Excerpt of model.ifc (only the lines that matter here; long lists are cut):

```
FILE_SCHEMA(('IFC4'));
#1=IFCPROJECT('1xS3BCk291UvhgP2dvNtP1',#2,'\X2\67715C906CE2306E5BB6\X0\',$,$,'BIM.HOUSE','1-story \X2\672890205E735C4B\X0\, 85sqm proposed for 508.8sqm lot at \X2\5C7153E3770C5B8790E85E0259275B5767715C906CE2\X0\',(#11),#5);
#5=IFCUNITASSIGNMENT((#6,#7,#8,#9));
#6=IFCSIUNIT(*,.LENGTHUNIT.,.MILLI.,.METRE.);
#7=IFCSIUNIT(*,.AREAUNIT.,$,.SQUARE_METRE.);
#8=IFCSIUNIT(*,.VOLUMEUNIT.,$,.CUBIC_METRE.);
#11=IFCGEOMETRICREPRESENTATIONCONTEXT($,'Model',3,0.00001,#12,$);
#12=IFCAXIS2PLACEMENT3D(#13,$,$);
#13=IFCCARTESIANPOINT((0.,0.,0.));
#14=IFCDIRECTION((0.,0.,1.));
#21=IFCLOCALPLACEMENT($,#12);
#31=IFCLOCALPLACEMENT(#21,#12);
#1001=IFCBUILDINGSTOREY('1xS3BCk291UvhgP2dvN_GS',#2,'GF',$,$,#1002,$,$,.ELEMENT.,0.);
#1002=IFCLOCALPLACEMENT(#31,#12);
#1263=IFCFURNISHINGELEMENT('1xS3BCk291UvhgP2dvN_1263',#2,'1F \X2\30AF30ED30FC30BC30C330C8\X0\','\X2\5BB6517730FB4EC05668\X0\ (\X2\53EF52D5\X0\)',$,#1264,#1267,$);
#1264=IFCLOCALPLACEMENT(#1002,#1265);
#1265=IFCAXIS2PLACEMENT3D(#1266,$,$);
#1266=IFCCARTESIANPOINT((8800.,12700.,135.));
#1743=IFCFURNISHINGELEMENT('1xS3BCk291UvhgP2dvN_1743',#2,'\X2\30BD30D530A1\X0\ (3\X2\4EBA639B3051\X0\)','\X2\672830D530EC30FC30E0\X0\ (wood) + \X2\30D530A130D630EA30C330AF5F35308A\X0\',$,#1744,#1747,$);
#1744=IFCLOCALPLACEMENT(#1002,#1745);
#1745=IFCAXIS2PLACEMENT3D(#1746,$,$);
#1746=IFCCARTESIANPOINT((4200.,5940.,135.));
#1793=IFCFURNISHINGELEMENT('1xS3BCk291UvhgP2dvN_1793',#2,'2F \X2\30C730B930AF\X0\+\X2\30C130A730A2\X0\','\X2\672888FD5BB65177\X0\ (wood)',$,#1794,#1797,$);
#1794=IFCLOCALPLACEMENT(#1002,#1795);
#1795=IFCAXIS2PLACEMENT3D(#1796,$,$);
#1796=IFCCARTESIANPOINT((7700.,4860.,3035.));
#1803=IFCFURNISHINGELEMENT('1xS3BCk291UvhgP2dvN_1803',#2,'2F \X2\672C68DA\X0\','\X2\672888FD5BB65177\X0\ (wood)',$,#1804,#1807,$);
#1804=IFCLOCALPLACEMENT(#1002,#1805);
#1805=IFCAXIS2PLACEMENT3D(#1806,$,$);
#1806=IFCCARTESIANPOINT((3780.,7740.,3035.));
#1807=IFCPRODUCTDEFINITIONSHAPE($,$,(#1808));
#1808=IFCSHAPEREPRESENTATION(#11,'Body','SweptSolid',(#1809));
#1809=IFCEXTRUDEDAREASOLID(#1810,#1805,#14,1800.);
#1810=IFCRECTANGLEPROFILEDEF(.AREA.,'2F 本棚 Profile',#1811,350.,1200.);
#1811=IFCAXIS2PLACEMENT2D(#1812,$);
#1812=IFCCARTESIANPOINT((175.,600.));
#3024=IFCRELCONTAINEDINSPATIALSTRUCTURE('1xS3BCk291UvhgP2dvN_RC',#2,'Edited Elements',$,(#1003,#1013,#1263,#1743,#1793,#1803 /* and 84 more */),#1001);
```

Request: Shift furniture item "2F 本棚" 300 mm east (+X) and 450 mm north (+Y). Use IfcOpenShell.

```python
import ifcopenshell
import ifcopenshell.api.geometry
import ifcopenshell.util.placement
import ifcopenshell.util.unit

model = ifcopenshell.open("model.ifc")
unit_scale = ifcopenshell.util.unit.calculate_unit_scale(model)

item = model.by_guid("1xS3BCk291UvhgP2dvN_1803")
matrix = ifcopenshell.util.placement.get_local_placement(item.ObjectPlacement)
matrix[0, 3] += 0.3 / unit_scale
matrix[1, 3] += 0.45 / unit_scale
ifcopenshell.api.geometry.edit_object_placement(model, product=item, matrix=matrix, is_si=False)

print(ifcopenshell.util.placement.get_local_placement(item.ObjectPlacement).round(3) + 0.0)

model.write("model-out.ifc")
```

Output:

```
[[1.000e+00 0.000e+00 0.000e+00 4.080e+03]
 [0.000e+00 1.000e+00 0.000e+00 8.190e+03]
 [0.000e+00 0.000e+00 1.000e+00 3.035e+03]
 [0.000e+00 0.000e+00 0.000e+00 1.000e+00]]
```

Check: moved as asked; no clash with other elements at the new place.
